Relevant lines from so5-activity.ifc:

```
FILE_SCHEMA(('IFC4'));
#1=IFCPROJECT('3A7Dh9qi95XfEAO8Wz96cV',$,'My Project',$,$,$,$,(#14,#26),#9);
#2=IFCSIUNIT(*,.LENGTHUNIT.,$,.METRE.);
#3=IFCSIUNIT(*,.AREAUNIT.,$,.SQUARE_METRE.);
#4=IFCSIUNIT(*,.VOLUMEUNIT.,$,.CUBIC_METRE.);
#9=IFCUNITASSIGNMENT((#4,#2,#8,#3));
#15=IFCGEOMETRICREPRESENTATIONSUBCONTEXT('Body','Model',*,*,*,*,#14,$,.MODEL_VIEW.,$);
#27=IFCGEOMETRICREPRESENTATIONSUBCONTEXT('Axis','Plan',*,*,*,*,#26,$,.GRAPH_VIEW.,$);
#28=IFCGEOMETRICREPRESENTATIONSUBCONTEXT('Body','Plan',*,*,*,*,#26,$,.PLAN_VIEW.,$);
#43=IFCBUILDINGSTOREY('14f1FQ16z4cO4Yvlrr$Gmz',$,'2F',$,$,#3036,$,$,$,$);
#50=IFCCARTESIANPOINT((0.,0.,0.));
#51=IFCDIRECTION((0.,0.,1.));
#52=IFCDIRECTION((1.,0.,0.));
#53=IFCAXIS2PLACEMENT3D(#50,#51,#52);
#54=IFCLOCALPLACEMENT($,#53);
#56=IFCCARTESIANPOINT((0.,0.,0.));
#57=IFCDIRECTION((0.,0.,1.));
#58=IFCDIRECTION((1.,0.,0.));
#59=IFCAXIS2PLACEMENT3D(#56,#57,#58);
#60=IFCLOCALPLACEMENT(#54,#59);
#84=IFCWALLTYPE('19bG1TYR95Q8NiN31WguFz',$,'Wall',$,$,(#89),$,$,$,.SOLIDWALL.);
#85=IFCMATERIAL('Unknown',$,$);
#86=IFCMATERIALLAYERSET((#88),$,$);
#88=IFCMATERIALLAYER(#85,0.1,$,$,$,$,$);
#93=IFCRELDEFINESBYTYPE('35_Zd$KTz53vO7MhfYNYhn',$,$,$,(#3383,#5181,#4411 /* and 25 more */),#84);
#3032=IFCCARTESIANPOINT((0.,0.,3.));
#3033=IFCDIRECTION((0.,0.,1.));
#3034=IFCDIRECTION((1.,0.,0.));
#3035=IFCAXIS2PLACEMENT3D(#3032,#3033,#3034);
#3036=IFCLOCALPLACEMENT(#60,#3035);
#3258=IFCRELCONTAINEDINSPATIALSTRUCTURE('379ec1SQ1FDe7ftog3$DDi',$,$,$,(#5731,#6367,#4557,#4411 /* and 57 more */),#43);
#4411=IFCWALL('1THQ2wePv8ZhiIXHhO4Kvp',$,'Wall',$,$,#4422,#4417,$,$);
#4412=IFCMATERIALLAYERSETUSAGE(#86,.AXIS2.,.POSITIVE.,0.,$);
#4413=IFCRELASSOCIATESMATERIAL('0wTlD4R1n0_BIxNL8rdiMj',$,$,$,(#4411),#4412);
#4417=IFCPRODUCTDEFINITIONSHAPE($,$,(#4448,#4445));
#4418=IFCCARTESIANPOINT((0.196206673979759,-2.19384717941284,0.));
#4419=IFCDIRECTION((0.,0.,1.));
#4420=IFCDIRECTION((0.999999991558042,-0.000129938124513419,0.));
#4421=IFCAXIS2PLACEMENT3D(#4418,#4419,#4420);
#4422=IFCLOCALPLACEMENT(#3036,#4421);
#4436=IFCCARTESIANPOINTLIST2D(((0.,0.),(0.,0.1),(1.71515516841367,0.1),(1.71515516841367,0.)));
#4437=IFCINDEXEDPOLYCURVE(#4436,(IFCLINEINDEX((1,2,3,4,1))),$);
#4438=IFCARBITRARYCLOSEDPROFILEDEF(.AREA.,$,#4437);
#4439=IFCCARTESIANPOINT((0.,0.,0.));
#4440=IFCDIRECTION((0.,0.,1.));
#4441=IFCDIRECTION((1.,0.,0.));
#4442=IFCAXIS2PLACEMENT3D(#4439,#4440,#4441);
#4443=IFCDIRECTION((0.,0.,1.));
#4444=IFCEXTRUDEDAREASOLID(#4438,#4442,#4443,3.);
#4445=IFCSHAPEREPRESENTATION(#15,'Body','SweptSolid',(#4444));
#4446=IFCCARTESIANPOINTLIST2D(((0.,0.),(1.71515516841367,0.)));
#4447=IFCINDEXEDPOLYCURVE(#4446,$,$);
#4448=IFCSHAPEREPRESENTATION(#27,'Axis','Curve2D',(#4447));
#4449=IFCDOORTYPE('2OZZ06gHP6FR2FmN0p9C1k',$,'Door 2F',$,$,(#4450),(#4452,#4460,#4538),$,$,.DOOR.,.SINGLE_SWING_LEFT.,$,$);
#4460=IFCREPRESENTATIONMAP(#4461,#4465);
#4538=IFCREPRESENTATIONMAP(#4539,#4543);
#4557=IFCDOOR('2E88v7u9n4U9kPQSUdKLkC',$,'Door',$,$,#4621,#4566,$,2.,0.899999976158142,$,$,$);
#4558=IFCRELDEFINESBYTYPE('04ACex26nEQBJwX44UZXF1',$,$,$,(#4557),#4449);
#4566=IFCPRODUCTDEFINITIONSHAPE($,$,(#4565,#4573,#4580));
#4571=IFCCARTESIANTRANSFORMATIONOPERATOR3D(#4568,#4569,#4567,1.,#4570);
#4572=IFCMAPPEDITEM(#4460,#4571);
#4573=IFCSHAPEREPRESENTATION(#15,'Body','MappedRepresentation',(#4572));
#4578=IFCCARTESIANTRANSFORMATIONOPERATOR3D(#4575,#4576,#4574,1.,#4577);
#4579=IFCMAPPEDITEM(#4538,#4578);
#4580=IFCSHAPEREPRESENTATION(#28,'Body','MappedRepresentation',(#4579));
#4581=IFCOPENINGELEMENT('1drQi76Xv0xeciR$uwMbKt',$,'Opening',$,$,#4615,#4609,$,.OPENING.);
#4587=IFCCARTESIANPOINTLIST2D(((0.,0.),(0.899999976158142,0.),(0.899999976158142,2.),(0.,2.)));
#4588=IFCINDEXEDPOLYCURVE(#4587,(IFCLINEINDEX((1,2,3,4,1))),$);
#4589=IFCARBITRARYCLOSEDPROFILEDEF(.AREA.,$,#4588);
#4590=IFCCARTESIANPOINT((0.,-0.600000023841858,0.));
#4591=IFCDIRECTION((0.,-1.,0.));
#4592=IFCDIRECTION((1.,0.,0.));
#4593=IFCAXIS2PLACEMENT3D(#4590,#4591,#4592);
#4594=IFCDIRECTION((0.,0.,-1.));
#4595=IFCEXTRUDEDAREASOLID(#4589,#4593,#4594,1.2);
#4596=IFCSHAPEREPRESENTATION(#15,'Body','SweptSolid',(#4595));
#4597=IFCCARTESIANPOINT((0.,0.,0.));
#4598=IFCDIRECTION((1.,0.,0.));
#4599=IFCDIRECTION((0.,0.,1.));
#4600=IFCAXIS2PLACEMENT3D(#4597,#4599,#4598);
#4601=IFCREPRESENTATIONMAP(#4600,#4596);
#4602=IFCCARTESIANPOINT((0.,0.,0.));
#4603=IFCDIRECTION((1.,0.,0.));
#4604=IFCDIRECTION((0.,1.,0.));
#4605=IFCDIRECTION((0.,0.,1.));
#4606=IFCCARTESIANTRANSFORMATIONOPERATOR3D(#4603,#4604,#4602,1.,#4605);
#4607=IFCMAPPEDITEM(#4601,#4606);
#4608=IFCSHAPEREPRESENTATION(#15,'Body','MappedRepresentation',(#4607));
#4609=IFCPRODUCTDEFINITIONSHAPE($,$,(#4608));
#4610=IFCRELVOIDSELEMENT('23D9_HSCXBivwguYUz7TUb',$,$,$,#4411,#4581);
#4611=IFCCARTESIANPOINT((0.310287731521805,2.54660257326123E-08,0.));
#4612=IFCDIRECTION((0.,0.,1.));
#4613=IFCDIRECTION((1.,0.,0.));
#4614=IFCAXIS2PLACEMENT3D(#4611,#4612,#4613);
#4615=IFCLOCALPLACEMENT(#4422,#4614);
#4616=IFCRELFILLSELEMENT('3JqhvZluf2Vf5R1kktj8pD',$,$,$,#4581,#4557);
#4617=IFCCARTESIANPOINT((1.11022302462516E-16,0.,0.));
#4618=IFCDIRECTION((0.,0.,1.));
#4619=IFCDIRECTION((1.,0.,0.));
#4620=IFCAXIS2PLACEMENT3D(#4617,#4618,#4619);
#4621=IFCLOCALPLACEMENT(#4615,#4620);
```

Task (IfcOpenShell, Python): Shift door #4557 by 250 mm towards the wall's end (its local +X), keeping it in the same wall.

```python
import ifcopenshell
import ifcopenshell.api.geometry
import ifcopenshell.util.placement

model = ifcopenshell.open("so5-activity.ifc")

door = model.by_id(4557)
opening = door.FillsVoids[0].RelatingOpeningElement
wall = opening.VoidsElements[0].RelatingBuildingElement

wall_matrix = ifcopenshell.util.placement.get_local_placement(wall.ObjectPlacement)
shift = wall_matrix[:3, 0] * 0.25
before = ifcopenshell.util.placement.get_local_placement(door.ObjectPlacement)[:3, 3].copy()

# The door is placed relative to its opening, so it follows when the opening moves.
matrix = ifcopenshell.util.placement.get_local_placement(opening.ObjectPlacement)
matrix[:3, 3] += shift
ifcopenshell.api.geometry.edit_object_placement(
    model, product=opening, matrix=matrix, is_si=False, should_transform_children=True
)

after = ifcopenshell.util.placement.get_local_placement(door.ObjectPlacement)[:3, 3]
print("door moved by", (after - before).round(3) + 0.0)

model.write("so5-activity_updated.ifc")
```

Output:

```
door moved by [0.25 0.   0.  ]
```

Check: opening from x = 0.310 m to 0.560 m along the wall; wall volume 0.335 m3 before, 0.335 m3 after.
